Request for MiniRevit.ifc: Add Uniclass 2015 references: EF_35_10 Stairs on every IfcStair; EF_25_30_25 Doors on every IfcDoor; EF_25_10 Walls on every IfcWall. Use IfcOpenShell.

First a look at what the model holds.

```python
import ifcopenshell

model = ifcopenshell.open("MiniRevit.ifc")
print(model.schema)
print("classifications:", [c.Name for c in model.by_type("IfcClassification")])
for ifc_class in ("IfcDoor", "IfcRoof", "IfcStair", "IfcWall", "IfcWindow"):
    print(ifc_class, len(model.by_type(ifc_class)))
```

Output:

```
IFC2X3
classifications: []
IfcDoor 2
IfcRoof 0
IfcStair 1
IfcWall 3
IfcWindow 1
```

```python
import ifcopenshell
import ifcopenshell.api.classification

model = ifcopenshell.open("MiniRevit.ifc")

# IFC2X3 requires Source and Edition and has no link from the project to the system.
system = model.create_entity("IfcClassification", Source="NBS", Edition="2015", Name="Uniclass 2015")

codes = {
    "IfcStair": ("EF_35_10", "Stairs"),
    "IfcDoor": ("EF_25_30_25", "Doors"),
    "IfcWall": ("EF_25_10", "Walls"),
}
for ifc_class, (code, name) in codes.items():
    products = model.by_type(ifc_class)
    ifcopenshell.api.classification.add_reference(
        model, products=products, classification=system, identification=code, name=name
    )
    print(code, len(products))

model.write("MiniRevit_v2.ifc")
```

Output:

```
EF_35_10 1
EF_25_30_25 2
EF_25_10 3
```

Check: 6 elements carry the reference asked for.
